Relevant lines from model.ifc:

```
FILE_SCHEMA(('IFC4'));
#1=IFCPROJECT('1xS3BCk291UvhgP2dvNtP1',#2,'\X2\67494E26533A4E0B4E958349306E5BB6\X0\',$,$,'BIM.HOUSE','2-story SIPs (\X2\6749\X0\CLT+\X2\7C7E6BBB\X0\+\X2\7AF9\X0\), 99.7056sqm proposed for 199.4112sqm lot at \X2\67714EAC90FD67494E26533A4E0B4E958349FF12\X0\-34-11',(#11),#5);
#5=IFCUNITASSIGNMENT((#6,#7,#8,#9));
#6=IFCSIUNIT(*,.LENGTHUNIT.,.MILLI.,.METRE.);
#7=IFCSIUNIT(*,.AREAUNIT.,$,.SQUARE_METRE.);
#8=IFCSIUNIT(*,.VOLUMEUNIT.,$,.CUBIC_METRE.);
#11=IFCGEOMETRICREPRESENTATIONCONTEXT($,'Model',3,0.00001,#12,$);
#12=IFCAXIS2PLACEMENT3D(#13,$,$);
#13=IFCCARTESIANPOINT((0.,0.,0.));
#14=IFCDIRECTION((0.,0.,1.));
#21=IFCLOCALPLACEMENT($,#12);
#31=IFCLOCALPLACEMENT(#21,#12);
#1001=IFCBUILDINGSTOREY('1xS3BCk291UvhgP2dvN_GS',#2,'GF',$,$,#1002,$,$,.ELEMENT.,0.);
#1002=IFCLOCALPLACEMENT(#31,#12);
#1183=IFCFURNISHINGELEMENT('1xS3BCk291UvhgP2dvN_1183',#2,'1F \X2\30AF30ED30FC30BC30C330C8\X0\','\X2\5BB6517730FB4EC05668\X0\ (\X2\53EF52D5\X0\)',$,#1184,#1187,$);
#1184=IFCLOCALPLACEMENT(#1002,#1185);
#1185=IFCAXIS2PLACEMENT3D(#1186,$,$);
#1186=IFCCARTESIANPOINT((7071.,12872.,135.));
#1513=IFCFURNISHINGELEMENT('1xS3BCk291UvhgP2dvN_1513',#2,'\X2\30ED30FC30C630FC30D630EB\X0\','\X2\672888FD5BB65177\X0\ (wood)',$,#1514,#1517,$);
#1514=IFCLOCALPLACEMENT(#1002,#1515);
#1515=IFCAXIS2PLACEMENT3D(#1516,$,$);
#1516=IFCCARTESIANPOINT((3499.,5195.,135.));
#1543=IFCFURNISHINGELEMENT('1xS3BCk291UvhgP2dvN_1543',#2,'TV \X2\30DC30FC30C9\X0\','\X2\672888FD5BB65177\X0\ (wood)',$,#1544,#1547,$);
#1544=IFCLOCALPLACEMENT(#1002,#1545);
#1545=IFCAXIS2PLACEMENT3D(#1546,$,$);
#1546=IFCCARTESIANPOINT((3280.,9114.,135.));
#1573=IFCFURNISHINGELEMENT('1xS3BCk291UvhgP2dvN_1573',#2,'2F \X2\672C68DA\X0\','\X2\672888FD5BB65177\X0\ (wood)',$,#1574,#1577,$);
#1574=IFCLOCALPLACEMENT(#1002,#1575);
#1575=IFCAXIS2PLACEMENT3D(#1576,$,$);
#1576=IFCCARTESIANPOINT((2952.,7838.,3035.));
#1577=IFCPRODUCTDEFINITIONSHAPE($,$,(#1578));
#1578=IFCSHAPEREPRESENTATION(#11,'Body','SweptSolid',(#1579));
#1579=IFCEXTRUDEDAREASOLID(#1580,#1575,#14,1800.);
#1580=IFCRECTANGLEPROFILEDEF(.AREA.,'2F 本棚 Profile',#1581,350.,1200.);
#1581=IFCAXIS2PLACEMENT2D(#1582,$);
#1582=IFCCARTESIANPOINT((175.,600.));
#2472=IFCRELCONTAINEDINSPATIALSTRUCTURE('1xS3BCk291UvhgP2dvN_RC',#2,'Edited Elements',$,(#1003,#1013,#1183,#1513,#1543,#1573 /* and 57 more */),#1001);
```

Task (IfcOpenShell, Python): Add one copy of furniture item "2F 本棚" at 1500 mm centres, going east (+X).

```python
import numpy as np
import ifcopenshell
import ifcopenshell.api.geometry
import ifcopenshell.api.root
import ifcopenshell.util.element
import ifcopenshell.util.placement
import ifcopenshell.util.unit

model = ifcopenshell.open("model.ifc")
unit_scale = ifcopenshell.util.unit.calculate_unit_scale(model)


def reuse_history(source, copy):
    """copy_class also copies each property set's owner history, people and application; keep the originals."""
    for rel in copy.IsDefinedBy:
        if rel.is_a("IfcRelDefinesByProperties") and (history := rel.RelatingPropertyDefinition.OwnerHistory):
            rel.RelatingPropertyDefinition.OwnerHistory = source.OwnerHistory
            ifcopenshell.util.element.remove_deep2(model, history)


source = model.by_guid("1xS3BCk291UvhgP2dvN_1573")
base = ifcopenshell.util.placement.get_local_placement(source.ObjectPlacement)
step = np.array([1.0, 0.0, 0.0]) * 1.5 / unit_scale

for i in range(1, 2):
    copy = ifcopenshell.api.root.copy_class(model, product=source)
    copy.Representation = ifcopenshell.util.element.copy_deep(
        model, source.Representation, exclude=["IfcGeometricRepresentationContext", "IfcRepresentationMap"]
    )
    reuse_history(source, copy)
    matrix = base.copy()
    matrix[:3, 3] += i * step
    print("added at", matrix[:3, 3].round(3) + 0.0)
    ifcopenshell.api.geometry.edit_object_placement(model, product=copy, matrix=matrix, is_si=False)

model.write("model_rev.ifc")
```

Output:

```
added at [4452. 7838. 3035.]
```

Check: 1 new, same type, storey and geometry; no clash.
